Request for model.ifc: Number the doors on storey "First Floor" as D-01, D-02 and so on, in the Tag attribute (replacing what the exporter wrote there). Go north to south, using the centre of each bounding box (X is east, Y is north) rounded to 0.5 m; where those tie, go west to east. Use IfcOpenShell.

First a look at what the model holds.

```python
import ifcopenshell
import ifcopenshell.util.element
import ifcopenshell.util.placement

model = ifcopenshell.open("model.ifc")
print(model.schema)
storey = next(s for s in model.by_type("IfcBuildingStorey") if s.Name == "First Floor")
doors = [e for e in ifcopenshell.util.element.get_decomposition(storey) if e.is_a("IfcDoor")]
for e in sorted(doors, key=lambda e: e.id()):
    origin = ifcopenshell.util.placement.get_local_placement(e.ObjectPlacement)[:3, 3]
    print(e.id(), e.Tag, e.Name, origin.round(2) + 0.0, sep=" | ")
```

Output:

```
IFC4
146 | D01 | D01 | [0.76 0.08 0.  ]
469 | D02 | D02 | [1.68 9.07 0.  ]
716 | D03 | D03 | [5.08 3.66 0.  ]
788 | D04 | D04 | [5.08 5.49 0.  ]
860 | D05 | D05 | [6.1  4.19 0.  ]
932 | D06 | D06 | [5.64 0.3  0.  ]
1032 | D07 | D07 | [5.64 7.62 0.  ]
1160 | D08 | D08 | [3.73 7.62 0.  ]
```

```python
import ifcopenshell
import ifcopenshell.geom
import ifcopenshell.util.element
import ifcopenshell.util.shape

model = ifcopenshell.open("model.ifc")
settings = ifcopenshell.geom.settings()
settings.set("use-world-coords", True)


def centre(element):
    shape = ifcopenshell.geom.create_shape(settings, element)
    return ifcopenshell.util.shape.get_bbox_centroid(shape.geometry)


storey = next(s for s in model.by_type("IfcBuildingStorey") if s.Name == "First Floor")
doors = [e for e in ifcopenshell.util.element.get_decomposition(storey) if e.is_a("IfcDoor")]

# Insertion points can sit at a corner or the storey origin, so sort by the geometry (in metres).
centres = {e: centre(e) for e in doors}
doors.sort(key=lambda e: (-round(centres[e][1] / 0.5), centres[e][0]))

for i, e in enumerate(doors, start=1):
    number = f"D-{i:02d}"
    e.Tag = number
    print(e.id(), number)

model.write("model_rev.ifc")
```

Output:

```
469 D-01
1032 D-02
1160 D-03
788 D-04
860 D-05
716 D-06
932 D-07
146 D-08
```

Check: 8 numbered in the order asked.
